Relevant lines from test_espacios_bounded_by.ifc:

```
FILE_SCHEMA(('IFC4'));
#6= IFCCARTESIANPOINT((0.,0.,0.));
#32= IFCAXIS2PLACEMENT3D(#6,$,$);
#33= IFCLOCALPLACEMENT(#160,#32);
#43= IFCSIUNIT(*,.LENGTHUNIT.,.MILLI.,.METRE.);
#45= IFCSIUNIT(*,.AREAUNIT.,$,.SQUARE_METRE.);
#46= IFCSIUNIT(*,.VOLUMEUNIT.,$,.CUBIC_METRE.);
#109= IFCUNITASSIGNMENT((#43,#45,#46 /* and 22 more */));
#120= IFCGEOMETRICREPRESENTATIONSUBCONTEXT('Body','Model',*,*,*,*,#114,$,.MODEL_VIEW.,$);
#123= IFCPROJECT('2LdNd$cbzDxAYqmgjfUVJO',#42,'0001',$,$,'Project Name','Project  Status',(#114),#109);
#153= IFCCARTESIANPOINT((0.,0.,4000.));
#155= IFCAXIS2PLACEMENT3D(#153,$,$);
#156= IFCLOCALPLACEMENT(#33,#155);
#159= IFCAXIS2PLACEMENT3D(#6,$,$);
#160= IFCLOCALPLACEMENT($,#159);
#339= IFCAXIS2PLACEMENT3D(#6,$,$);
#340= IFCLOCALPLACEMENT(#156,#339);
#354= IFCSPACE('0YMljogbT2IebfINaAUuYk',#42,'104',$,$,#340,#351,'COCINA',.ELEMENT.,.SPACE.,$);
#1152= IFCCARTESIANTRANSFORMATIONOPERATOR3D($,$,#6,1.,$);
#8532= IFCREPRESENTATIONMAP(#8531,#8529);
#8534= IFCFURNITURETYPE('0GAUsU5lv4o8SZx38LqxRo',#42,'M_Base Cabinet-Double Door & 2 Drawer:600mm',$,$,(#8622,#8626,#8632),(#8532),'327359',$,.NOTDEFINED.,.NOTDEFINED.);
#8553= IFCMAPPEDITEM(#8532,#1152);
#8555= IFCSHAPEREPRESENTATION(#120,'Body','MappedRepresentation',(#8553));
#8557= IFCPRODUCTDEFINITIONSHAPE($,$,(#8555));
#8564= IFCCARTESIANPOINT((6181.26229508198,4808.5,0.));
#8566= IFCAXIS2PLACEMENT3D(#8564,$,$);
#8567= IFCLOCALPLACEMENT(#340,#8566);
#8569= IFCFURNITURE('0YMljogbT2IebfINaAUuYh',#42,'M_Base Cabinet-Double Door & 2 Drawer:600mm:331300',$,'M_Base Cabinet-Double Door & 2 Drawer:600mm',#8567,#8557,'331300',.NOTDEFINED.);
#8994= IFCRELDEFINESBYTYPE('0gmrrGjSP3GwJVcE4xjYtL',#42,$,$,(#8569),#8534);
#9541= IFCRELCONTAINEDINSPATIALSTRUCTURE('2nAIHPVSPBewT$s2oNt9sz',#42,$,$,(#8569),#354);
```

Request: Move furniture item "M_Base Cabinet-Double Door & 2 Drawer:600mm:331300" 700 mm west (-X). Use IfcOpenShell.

```python
import ifcopenshell
import ifcopenshell.api.geometry
import ifcopenshell.util.placement
import ifcopenshell.util.unit

model = ifcopenshell.open("test_espacios_bounded_by.ifc")
unit_scale = ifcopenshell.util.unit.calculate_unit_scale(model)

item = model.by_guid("0YMljogbT2IebfINaAUuYh")
matrix = ifcopenshell.util.placement.get_local_placement(item.ObjectPlacement)
matrix[0, 3] -= 0.7 / unit_scale
ifcopenshell.api.geometry.edit_object_placement(model, product=item, matrix=matrix, is_si=False)

print(ifcopenshell.util.placement.get_local_placement(item.ObjectPlacement).round(3) + 0.0)

model.write("test_espacios_bounded_by-out.ifc")
```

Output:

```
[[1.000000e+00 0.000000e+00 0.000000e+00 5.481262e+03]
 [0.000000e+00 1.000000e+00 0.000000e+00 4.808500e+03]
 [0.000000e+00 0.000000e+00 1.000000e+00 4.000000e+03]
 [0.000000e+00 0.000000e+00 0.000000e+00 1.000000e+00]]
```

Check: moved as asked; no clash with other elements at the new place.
